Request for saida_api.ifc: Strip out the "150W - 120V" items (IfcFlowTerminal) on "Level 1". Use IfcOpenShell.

First a look at what the model holds.

```python
import ifcopenshell
import ifcopenshell.util.element

model = ifcopenshell.open("saida_api.ifc")
print(model.schema)
storey = next(s for s in model.by_type("IfcBuildingStorey") if s.Name == "Level 1")
terminals = [e for e in ifcopenshell.util.element.get_decomposition(storey) if e.is_a("IfcFlowTerminal")]
seen = {}
for e in terminals:
    element_type = ifcopenshell.util.element.get_type(e)
    name = element_type.Name if element_type not in (None, e) else None
    seen[name] = seen.get(name, 0) + 1
for name, count in sorted(seen.items(), key=str):
    print(count, "x", name)
```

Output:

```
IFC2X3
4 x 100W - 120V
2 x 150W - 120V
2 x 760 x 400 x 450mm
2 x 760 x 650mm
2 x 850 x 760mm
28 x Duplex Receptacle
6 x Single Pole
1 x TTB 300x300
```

```python
import ifcopenshell
import ifcopenshell.api.root
import ifcopenshell.util.element

model = ifcopenshell.open("saida_api.ifc")

storey = next(s for s in model.by_type("IfcBuildingStorey") if s.Name == "Level 1")
terminals = [e for e in ifcopenshell.util.element.get_decomposition(storey) if e.is_a("IfcFlowTerminal")]
targets = [e for e in terminals if (t := ifcopenshell.util.element.get_type(e)) not in (None, e) and t.Name == "150W - 120V"]

for e in targets:
    ifcopenshell.api.root.remove_product(model, product=e)
print(len(targets), "removed")

model.write("saida_api_v2.ifc")
```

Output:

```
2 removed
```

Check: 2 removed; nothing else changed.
